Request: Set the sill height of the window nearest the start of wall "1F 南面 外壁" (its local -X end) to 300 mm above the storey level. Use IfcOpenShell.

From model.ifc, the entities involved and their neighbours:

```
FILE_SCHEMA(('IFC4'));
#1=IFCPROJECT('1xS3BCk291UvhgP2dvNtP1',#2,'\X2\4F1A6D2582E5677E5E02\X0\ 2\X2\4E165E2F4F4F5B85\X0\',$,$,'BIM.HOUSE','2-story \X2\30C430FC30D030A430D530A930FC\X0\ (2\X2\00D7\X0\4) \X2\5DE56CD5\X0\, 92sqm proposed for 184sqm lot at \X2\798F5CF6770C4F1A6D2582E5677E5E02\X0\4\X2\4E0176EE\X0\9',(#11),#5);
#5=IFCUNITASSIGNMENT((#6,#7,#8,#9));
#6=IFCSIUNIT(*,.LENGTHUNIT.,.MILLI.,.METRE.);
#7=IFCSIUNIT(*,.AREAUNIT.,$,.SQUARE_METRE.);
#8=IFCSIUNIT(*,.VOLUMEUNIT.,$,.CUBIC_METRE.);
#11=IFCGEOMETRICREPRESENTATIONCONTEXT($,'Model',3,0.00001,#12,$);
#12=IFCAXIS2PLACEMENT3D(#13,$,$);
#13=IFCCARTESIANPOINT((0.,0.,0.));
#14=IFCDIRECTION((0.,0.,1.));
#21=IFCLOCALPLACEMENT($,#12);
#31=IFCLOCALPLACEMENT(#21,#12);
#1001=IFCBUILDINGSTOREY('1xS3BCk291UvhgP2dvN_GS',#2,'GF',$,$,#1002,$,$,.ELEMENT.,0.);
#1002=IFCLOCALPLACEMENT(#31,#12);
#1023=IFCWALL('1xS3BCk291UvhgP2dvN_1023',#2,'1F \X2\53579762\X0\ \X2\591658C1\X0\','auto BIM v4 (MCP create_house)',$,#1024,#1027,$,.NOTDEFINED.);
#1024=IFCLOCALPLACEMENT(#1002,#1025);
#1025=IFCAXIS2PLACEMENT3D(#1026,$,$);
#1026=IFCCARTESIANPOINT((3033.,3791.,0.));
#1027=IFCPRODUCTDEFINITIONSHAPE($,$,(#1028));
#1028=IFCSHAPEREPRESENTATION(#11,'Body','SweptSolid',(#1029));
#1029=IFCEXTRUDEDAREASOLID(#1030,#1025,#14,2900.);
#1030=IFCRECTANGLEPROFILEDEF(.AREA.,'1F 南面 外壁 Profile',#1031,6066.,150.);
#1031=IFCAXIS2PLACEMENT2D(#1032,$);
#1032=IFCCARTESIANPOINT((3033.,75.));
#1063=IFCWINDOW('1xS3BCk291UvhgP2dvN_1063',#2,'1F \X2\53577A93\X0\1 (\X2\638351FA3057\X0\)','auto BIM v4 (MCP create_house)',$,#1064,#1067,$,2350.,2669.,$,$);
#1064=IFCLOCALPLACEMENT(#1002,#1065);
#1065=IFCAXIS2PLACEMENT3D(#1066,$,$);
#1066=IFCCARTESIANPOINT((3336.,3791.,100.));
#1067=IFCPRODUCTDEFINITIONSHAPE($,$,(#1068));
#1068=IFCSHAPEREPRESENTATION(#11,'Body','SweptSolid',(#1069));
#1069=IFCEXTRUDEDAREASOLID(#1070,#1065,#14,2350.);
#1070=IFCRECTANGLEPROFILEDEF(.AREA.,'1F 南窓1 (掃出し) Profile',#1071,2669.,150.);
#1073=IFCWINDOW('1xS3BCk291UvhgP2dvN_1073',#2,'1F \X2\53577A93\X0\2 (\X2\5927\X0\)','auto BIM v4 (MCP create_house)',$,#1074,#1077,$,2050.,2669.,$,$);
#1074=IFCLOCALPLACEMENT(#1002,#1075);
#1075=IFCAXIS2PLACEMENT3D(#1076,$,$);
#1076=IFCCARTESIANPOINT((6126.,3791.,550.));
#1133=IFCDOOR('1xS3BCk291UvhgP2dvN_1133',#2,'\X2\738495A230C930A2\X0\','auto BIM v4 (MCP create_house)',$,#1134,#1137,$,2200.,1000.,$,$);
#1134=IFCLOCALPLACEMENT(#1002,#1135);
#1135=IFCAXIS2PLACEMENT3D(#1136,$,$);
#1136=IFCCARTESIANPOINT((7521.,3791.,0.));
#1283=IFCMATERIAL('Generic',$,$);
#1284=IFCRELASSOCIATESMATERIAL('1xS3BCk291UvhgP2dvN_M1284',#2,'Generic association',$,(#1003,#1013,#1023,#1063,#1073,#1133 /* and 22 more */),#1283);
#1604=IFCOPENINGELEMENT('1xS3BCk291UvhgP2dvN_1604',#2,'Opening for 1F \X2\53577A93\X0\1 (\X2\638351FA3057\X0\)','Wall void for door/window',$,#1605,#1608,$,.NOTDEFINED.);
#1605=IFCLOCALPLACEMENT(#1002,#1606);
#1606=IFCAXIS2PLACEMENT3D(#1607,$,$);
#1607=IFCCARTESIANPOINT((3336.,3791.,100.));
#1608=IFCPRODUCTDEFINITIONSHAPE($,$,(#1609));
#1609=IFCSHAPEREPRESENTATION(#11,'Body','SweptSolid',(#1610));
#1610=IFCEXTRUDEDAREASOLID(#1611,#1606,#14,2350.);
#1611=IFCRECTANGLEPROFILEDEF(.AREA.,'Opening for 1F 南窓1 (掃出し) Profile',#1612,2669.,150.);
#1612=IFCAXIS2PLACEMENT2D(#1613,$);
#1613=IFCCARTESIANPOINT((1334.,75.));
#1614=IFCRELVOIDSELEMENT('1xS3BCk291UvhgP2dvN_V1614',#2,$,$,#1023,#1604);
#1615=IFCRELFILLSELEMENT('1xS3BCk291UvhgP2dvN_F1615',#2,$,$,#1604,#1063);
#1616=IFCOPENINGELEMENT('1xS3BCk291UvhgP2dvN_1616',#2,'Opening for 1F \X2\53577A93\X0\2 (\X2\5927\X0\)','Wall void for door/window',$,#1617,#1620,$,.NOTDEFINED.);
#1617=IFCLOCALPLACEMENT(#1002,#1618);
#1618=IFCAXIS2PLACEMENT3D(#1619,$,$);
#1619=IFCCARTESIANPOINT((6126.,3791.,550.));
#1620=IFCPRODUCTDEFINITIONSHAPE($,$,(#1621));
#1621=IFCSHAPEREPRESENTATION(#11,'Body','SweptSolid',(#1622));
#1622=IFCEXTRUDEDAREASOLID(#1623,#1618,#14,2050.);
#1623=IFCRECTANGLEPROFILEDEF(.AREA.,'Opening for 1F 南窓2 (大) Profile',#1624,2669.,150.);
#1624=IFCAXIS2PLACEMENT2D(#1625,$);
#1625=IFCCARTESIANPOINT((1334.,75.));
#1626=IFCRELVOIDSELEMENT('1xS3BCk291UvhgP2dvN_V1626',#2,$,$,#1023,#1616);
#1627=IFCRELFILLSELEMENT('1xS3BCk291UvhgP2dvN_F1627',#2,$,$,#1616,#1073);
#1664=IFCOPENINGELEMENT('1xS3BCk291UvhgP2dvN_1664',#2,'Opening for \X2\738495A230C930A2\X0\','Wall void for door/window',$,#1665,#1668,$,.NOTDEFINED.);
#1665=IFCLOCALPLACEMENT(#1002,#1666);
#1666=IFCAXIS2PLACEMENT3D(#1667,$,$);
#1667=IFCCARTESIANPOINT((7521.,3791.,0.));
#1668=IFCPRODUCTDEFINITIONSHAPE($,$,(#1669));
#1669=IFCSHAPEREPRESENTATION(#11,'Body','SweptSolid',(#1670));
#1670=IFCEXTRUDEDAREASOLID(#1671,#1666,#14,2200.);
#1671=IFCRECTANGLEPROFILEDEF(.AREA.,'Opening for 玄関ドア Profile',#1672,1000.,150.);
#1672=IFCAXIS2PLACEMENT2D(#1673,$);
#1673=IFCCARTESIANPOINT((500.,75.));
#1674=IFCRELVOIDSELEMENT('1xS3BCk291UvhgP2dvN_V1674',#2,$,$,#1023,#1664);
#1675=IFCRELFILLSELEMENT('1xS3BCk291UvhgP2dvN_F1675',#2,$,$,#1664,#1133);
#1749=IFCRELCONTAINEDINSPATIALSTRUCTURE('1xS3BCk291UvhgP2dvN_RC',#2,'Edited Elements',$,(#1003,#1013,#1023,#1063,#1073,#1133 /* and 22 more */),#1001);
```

```python
import numpy as np
import ifcopenshell
import ifcopenshell.api.geometry
import ifcopenshell.geom
import ifcopenshell.util.element
import ifcopenshell.util.placement
import ifcopenshell.util.shape
import ifcopenshell.util.unit

model = ifcopenshell.open("model.ifc")
unit_scale = ifcopenshell.util.unit.calculate_unit_scale(model)

window = model.by_guid("1xS3BCk291UvhgP2dvN_1063")
opening = window.FillsVoids[0].RelatingOpeningElement
storey = ifcopenshell.util.element.get_container(window, ifc_class="IfcBuildingStorey")
level = ifcopenshell.util.placement.get_local_placement(storey.ObjectPlacement)[2, 3]

# The opening's origin need not be at the sill, so measure its lowest point.
shape = ifcopenshell.geom.create_shape(ifcopenshell.geom.settings(), opening)
bottom = ifcopenshell.util.shape.get_shape_bottom_elevation(shape, shape.geometry) / unit_scale
dz = level + 0.3 / unit_scale - bottom

shift = np.array([0.0, 0.0, dz])
# The window is not placed relative to its opening, so move both.
for product in (opening, window):
    matrix = ifcopenshell.util.placement.get_local_placement(product.ObjectPlacement)
    matrix[:3, 3] += shift
    ifcopenshell.api.geometry.edit_object_placement(model, product=product, matrix=matrix, is_si=False)

print(f"moved by {dz * unit_scale:+.3f} m")

model.write("model_edited.ifc")
```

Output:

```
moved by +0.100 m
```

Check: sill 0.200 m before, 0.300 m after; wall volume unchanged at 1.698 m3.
